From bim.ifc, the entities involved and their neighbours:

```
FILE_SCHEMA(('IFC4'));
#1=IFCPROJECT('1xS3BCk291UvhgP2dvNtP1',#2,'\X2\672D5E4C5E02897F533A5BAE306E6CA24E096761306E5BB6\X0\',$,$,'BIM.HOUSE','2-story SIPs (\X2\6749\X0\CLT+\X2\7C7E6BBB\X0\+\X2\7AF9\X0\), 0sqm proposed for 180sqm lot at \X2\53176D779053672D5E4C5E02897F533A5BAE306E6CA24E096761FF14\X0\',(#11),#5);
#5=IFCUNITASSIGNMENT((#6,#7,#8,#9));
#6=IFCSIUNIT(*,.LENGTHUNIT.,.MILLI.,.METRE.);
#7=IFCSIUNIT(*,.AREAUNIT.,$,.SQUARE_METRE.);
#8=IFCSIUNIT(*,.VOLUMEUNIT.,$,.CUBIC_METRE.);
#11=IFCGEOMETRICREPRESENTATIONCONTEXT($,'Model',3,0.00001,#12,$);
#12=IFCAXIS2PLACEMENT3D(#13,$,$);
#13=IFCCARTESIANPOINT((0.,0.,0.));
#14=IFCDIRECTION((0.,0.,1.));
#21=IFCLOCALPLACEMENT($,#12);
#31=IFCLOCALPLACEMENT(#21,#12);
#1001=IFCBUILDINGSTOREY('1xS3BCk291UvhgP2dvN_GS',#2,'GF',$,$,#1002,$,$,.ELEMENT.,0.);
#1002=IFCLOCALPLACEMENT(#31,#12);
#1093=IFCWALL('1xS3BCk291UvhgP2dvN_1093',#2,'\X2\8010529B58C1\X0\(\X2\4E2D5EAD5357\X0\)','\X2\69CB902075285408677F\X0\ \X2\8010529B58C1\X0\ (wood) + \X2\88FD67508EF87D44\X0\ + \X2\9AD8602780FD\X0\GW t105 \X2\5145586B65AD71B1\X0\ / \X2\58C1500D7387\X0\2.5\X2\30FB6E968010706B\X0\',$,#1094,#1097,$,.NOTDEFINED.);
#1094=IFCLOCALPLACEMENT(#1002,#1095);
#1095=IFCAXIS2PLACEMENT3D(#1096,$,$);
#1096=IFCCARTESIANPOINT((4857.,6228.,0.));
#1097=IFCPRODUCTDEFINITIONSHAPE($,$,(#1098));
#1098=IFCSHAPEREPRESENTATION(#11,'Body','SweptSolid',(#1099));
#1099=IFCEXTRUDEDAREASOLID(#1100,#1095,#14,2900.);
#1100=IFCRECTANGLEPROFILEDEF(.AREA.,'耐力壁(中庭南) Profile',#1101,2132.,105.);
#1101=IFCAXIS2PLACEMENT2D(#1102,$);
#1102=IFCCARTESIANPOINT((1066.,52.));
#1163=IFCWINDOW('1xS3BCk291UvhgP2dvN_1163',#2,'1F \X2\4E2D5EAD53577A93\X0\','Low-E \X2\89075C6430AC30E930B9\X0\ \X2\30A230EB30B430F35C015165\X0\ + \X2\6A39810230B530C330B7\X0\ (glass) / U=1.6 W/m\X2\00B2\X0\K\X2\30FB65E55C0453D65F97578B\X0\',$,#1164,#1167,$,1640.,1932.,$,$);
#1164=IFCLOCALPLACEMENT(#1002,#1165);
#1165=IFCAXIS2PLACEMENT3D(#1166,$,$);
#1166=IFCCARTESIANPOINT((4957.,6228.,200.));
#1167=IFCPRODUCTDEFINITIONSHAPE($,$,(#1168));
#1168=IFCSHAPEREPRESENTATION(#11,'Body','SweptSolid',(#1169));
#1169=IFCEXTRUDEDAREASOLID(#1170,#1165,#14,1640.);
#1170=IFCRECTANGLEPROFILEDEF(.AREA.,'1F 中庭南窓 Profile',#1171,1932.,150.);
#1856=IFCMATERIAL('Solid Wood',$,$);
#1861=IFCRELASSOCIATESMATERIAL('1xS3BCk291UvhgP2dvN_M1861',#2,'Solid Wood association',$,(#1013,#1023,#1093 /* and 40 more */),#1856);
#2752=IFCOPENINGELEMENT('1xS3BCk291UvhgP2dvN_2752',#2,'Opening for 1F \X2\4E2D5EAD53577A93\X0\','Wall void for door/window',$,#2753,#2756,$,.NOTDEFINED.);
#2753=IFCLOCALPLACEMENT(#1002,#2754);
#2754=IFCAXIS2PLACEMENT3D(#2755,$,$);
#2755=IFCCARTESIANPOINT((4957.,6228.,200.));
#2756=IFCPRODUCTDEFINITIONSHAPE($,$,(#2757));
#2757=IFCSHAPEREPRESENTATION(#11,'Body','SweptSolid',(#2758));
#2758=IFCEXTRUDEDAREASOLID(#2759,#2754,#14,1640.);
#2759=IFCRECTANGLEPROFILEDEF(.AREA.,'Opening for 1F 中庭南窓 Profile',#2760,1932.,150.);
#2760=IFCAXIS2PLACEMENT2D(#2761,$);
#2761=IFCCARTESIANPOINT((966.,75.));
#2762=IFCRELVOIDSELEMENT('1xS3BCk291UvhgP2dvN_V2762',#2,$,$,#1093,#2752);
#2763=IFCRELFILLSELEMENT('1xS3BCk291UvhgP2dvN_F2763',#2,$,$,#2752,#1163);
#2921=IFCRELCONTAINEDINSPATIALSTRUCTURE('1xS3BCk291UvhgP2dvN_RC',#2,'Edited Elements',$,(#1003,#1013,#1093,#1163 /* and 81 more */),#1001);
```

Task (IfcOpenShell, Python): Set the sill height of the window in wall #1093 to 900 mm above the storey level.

```python
import numpy as np
import ifcopenshell
import ifcopenshell.api.geometry
import ifcopenshell.geom
import ifcopenshell.util.element
import ifcopenshell.util.placement
import ifcopenshell.util.shape
import ifcopenshell.util.unit

model = ifcopenshell.open("bim.ifc")
unit_scale = ifcopenshell.util.unit.calculate_unit_scale(model)

window = model.by_guid("1xS3BCk291UvhgP2dvN_1163")
opening = window.FillsVoids[0].RelatingOpeningElement
storey = ifcopenshell.util.element.get_container(window, ifc_class="IfcBuildingStorey")
level = ifcopenshell.util.placement.get_local_placement(storey.ObjectPlacement)[2, 3]

# The opening's origin need not be at the sill, so measure its lowest point.
shape = ifcopenshell.geom.create_shape(ifcopenshell.geom.settings(), opening)
bottom = ifcopenshell.util.shape.get_shape_bottom_elevation(shape, shape.geometry) / unit_scale
dz = level + 0.9 / unit_scale - bottom

shift = np.array([0.0, 0.0, dz])
# The window is not placed relative to its opening, so move both.
for product in (opening, window):
    matrix = ifcopenshell.util.placement.get_local_placement(product.ObjectPlacement)
    matrix[:3, 3] += shift
    ifcopenshell.api.geometry.edit_object_placement(model, product=product, matrix=matrix, is_si=False)

print(f"moved by {dz * unit_scale:+.3f} m")

model.write("bim_v2.ifc")
```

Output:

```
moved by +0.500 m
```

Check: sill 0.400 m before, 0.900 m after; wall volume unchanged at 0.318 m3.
